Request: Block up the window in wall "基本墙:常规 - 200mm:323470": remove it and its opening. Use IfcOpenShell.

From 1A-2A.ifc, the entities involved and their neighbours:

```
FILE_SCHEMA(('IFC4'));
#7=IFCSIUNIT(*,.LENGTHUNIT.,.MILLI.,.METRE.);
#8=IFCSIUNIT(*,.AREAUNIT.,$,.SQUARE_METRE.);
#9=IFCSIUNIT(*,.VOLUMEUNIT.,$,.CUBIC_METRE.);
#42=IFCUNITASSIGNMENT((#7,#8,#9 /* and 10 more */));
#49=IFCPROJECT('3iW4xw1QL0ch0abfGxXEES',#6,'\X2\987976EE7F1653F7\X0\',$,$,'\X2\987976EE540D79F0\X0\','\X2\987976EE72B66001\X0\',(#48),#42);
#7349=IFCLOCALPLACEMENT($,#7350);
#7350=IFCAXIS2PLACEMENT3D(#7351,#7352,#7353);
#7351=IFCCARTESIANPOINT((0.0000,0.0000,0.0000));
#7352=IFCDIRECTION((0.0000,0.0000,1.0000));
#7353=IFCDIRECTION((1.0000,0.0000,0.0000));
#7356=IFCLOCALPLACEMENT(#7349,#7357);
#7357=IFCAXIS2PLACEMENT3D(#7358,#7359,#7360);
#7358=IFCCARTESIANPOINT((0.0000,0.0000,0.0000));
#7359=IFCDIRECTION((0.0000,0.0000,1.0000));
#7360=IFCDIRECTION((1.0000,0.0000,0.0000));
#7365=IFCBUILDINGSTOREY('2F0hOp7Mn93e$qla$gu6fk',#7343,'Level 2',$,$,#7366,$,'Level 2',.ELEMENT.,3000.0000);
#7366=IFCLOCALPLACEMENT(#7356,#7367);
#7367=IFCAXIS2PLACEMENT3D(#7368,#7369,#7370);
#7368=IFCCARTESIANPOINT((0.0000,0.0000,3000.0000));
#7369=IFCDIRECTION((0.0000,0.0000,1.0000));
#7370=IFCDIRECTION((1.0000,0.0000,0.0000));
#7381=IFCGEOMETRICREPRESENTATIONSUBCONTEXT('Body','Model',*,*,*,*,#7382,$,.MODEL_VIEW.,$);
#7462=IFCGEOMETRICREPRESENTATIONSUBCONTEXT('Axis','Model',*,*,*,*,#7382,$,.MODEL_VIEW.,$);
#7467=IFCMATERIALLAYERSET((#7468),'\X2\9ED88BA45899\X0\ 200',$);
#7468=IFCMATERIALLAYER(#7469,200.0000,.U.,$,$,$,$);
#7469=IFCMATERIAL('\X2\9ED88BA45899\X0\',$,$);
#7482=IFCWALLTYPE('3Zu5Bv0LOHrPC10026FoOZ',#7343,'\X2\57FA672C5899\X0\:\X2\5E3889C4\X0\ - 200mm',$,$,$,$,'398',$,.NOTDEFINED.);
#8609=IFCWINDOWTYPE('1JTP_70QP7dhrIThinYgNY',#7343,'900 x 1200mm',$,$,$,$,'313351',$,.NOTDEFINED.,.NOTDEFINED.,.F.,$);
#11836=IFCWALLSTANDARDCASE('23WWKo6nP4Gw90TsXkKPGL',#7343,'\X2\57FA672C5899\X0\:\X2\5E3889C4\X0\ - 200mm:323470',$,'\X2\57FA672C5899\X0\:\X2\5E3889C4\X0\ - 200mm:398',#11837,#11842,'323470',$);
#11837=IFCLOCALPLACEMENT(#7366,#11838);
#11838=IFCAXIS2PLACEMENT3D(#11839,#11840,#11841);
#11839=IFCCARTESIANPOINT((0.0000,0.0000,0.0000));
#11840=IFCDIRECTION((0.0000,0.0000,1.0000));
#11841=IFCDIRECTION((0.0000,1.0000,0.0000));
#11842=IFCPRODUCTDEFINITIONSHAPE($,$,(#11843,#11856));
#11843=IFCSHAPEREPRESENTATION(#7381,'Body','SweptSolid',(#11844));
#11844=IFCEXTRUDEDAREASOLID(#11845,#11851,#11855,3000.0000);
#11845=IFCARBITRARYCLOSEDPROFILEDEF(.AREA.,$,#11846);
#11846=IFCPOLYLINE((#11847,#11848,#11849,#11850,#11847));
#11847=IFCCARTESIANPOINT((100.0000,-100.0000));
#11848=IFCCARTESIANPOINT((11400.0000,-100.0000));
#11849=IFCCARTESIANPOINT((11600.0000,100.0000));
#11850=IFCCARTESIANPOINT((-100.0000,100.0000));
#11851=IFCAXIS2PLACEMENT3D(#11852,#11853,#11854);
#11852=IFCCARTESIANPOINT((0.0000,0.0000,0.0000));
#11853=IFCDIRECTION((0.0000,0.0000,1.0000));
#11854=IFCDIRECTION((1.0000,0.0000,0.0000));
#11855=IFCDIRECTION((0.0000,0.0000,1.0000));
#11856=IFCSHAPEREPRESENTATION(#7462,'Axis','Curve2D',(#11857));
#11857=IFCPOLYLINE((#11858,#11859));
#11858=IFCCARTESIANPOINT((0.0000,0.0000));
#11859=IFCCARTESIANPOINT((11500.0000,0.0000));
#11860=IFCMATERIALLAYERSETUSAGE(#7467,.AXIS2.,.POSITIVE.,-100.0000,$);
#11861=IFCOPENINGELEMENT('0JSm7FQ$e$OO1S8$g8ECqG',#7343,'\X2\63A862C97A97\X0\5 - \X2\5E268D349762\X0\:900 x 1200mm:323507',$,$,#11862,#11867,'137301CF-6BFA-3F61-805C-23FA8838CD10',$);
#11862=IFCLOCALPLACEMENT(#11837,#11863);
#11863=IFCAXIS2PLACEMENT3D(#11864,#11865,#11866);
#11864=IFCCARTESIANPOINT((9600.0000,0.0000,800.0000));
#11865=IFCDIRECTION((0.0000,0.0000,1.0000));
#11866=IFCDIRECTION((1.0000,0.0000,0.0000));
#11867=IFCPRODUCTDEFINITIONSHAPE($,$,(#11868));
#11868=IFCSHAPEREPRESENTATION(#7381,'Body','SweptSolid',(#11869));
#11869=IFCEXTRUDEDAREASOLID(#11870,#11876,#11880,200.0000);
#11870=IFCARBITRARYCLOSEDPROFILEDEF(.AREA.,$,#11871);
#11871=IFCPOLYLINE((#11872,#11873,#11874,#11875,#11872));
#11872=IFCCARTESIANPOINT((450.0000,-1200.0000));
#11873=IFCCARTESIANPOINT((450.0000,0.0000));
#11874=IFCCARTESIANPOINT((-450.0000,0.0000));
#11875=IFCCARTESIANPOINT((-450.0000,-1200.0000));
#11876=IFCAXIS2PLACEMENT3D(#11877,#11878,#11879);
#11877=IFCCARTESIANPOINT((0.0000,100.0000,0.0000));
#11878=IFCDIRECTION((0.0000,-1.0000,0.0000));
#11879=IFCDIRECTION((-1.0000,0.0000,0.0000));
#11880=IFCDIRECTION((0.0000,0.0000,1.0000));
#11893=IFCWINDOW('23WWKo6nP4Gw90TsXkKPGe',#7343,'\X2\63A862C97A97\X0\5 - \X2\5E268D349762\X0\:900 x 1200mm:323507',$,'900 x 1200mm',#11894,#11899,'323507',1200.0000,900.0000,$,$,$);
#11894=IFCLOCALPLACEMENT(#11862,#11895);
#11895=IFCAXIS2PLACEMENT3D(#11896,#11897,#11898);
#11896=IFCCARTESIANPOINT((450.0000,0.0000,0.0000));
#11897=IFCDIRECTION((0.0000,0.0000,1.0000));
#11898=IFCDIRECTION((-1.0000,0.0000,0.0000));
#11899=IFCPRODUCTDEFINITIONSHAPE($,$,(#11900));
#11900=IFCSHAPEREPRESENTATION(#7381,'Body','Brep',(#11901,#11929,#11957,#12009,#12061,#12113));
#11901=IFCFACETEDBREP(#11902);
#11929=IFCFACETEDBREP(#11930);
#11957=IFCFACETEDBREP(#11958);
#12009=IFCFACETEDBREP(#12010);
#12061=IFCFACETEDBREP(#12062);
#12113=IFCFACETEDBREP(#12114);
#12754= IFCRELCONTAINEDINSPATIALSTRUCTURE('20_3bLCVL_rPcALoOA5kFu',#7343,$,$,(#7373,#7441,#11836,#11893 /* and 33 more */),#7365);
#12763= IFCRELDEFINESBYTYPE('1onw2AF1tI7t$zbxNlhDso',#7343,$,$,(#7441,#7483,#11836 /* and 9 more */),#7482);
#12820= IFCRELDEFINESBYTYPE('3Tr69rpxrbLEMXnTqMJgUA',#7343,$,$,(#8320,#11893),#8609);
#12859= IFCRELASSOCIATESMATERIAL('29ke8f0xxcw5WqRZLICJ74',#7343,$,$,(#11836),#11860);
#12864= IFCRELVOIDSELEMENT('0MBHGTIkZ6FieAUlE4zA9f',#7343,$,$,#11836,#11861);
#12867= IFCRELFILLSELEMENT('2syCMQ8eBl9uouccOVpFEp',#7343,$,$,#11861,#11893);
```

```python
import ifcopenshell
import ifcopenshell.api.feature
import ifcopenshell.api.root
import ifcopenshell.geom
import ifcopenshell.util.shape

model = ifcopenshell.open("1A-2A.ifc")
settings = ifcopenshell.geom.settings()


def volume(element):
    """Net volume in cubic metres, openings subtracted."""
    shape = ifcopenshell.geom.create_shape(settings, element)
    return ifcopenshell.util.shape.get_volume(shape.geometry)


window = model.by_id(11893)
opening = window.FillsVoids[0].RelatingOpeningElement
wall = opening.VoidsElements[0].RelatingBuildingElement
before = volume(wall)

ifcopenshell.api.root.remove_product(model, product=window)
ifcopenshell.api.feature.remove_feature(model, feature=opening)

after = volume(wall)

print(f"wall volume {before:.3f} -> {after:.3f} m3")

model.write("1A-2A_updated.ifc")
```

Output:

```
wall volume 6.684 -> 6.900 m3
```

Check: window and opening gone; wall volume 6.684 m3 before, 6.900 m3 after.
